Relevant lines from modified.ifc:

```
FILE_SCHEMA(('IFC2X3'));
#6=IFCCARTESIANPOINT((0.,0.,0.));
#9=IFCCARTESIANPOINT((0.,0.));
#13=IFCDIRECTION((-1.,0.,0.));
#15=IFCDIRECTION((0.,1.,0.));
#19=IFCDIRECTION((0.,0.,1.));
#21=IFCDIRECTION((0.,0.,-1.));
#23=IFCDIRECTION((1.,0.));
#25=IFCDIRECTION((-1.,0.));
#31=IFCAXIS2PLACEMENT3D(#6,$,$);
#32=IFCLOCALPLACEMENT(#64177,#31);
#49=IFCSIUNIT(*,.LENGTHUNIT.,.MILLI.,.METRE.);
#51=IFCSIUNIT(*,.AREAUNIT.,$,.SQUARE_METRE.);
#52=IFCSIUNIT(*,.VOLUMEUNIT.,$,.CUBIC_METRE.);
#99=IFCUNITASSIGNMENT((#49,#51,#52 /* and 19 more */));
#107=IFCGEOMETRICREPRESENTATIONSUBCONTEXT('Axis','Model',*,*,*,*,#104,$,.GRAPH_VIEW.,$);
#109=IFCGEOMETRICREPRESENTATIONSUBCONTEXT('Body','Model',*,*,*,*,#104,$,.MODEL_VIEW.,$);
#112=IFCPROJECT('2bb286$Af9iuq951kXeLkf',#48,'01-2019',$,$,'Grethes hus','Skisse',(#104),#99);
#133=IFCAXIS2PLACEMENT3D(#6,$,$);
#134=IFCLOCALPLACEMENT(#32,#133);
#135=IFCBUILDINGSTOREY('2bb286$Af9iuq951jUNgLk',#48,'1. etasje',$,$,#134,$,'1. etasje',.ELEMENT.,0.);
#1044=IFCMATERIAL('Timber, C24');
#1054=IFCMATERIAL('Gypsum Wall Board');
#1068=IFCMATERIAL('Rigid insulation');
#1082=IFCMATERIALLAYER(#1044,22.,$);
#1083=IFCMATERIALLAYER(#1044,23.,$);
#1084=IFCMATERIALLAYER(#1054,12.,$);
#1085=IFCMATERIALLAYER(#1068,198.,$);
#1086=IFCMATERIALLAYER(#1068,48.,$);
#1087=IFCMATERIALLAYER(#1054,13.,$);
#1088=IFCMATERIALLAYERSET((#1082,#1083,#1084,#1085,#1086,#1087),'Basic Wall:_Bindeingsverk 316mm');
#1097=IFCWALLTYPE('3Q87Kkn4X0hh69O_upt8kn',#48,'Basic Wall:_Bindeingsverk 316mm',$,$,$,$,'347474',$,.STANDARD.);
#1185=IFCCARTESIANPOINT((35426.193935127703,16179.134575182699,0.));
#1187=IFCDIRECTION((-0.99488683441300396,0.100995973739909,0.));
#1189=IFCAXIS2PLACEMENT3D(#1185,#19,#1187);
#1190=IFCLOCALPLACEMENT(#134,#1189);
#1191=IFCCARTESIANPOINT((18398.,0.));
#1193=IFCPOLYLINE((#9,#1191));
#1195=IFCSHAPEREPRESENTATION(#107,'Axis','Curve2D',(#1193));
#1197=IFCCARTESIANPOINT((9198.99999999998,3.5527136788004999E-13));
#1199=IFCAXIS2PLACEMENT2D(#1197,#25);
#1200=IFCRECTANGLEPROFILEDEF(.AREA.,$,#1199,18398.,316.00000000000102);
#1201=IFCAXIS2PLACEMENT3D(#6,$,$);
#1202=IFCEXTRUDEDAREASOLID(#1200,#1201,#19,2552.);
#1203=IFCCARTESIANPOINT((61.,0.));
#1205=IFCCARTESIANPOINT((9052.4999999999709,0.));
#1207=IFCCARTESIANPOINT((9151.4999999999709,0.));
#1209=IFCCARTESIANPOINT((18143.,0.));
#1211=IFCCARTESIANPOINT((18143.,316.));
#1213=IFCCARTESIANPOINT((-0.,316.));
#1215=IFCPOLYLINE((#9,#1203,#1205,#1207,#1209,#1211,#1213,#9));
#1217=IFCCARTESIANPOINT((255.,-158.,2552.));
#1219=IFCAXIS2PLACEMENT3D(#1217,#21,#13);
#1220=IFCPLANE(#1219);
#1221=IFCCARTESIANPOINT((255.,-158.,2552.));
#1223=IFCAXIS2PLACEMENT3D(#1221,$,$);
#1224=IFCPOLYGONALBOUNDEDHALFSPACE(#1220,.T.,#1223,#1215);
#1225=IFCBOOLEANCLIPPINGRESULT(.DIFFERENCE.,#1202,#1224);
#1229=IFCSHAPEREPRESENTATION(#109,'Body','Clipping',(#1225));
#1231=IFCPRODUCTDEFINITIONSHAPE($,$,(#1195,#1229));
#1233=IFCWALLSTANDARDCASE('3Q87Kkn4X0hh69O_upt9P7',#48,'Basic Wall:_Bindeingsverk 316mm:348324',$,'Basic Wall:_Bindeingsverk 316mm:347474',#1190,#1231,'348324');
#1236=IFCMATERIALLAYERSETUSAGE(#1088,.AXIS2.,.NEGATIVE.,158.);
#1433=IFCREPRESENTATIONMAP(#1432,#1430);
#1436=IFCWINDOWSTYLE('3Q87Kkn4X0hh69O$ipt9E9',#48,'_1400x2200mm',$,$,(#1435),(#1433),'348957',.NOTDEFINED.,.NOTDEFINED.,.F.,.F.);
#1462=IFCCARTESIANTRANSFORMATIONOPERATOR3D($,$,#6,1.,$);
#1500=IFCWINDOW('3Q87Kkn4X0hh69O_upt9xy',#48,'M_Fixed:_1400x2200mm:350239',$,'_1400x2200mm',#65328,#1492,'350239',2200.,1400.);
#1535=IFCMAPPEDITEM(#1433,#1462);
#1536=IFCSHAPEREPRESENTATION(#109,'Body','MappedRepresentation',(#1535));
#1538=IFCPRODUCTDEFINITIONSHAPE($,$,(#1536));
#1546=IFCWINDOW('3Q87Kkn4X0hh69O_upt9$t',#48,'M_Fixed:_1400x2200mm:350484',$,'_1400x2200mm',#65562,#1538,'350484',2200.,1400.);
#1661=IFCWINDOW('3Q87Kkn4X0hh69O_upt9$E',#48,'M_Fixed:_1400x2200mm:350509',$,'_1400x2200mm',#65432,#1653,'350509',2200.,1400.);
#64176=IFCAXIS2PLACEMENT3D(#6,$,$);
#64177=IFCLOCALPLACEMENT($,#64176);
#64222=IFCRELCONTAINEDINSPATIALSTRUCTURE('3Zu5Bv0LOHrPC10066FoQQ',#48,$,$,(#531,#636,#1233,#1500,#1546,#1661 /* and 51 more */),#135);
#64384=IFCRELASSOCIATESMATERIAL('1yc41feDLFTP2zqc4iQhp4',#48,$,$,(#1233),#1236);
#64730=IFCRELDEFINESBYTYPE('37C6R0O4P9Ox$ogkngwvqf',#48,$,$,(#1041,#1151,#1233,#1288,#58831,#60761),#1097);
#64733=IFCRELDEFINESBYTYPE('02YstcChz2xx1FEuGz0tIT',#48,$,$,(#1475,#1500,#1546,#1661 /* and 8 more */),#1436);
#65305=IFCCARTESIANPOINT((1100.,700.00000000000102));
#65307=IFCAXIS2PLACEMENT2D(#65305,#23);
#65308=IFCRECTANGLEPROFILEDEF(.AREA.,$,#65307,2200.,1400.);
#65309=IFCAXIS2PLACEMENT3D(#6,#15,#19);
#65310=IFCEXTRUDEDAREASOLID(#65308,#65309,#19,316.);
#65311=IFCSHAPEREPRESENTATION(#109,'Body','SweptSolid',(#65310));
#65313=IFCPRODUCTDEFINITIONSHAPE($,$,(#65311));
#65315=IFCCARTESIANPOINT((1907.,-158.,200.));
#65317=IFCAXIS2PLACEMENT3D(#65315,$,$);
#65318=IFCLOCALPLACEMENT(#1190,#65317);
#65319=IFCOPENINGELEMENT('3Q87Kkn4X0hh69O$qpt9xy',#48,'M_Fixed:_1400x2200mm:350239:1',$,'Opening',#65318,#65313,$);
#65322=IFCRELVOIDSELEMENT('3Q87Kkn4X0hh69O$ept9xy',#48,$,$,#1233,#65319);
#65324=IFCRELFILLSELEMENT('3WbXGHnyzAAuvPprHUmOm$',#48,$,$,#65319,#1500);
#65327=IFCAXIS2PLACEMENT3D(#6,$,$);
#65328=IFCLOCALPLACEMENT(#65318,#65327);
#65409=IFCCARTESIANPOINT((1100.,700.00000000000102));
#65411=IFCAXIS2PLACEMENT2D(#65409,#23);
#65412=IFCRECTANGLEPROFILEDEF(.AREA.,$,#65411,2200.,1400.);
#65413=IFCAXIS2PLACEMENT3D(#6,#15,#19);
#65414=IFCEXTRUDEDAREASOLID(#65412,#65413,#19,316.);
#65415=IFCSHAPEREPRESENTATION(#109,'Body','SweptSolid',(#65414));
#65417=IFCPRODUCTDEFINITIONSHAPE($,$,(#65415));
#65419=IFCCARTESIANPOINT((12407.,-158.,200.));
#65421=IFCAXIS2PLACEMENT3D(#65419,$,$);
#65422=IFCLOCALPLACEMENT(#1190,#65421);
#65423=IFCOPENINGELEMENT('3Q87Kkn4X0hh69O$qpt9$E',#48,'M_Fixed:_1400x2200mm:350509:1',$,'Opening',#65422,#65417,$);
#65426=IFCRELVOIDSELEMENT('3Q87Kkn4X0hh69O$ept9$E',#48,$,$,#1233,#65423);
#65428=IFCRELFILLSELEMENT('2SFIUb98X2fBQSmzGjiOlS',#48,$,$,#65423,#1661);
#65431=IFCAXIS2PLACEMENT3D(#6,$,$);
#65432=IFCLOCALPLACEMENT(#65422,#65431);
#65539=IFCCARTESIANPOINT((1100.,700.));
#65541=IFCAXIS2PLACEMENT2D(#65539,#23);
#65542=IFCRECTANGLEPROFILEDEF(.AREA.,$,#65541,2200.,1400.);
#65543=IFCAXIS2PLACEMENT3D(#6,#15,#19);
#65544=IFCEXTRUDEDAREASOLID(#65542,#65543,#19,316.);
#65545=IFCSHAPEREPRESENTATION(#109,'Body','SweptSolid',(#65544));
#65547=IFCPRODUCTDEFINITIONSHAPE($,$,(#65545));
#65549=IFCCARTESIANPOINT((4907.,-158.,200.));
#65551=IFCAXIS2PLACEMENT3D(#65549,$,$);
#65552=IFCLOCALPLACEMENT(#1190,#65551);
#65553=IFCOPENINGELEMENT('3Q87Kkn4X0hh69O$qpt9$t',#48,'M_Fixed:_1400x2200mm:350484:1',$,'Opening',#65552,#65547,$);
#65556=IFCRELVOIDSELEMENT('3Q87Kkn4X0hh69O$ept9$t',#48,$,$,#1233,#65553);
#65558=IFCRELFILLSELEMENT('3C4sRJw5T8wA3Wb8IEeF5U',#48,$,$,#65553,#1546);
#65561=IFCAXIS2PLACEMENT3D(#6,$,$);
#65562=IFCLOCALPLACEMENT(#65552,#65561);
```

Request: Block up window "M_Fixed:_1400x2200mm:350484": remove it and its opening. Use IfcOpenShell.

```python
import ifcopenshell
import ifcopenshell.api.feature
import ifcopenshell.api.root
import ifcopenshell.geom
import ifcopenshell.util.shape

model = ifcopenshell.open("modified.ifc")
settings = ifcopenshell.geom.settings()


def volume(element):
    """Net volume in cubic metres, openings subtracted."""
    shape = ifcopenshell.geom.create_shape(settings, element)
    return ifcopenshell.util.shape.get_volume(shape.geometry)


window = model.by_guid("3Q87Kkn4X0hh69O_upt9$t")
opening = window.FillsVoids[0].RelatingOpeningElement
wall = opening.VoidsElements[0].RelatingBuildingElement
before = volume(wall)

ifcopenshell.api.root.remove_product(model, product=window)
ifcopenshell.api.feature.remove_feature(model, feature=opening)

after = volume(wall)

print(f"wall volume {before:.3f} -> {after:.3f} m3")

model.write("modified_edited.ifc")
```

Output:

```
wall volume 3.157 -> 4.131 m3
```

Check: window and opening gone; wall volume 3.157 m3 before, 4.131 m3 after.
